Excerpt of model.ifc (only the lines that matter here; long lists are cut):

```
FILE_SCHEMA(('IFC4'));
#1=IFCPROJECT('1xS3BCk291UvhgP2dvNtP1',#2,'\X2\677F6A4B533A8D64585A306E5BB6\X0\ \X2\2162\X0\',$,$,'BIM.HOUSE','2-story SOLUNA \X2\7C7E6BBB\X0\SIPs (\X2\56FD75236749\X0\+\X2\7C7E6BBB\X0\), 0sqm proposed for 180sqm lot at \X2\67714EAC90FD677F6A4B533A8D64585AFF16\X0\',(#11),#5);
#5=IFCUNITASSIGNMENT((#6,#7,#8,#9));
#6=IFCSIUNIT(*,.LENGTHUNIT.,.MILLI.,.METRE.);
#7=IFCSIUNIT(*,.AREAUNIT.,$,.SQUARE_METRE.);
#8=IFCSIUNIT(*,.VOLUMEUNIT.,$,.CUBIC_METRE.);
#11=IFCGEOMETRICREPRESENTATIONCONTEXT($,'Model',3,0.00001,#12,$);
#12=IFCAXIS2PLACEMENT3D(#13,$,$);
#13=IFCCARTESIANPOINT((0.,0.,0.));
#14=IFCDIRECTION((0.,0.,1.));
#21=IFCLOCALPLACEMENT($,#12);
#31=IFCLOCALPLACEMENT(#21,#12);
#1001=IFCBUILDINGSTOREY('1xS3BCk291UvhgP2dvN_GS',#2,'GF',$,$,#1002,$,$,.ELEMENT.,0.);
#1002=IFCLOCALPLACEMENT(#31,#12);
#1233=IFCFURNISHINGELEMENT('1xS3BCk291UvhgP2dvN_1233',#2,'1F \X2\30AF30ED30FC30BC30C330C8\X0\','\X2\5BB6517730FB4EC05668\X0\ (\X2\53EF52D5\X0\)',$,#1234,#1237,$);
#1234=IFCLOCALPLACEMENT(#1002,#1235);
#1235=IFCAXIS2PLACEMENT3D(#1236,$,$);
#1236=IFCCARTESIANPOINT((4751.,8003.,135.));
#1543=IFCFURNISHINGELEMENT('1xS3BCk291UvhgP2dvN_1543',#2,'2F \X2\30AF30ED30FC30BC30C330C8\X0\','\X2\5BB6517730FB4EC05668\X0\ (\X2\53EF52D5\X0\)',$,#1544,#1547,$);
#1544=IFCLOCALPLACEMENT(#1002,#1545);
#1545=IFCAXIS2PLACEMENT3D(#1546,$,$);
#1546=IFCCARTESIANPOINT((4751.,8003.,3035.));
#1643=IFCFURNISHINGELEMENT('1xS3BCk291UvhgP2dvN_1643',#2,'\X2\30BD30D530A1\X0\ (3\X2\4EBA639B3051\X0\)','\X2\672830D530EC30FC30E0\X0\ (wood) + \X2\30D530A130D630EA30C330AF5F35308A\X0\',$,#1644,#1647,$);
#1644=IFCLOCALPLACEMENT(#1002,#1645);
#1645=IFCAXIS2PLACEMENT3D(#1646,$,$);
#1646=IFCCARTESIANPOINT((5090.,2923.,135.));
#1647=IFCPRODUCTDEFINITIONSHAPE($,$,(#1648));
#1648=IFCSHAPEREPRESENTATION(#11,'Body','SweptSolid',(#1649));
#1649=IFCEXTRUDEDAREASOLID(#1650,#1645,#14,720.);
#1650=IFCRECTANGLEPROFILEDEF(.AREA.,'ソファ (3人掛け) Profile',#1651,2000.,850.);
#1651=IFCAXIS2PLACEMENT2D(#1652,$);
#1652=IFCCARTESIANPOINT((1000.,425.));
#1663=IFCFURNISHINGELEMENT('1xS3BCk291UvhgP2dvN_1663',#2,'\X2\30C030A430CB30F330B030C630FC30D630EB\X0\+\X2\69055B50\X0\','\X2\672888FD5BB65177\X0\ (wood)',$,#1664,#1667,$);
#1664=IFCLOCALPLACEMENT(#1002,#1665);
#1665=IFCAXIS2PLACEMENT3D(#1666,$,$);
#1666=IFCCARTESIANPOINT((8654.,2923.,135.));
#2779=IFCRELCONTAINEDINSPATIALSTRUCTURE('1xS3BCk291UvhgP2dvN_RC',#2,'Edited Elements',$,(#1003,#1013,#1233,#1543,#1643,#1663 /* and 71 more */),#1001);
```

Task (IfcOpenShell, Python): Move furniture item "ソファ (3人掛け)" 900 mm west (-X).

```python
import ifcopenshell
import ifcopenshell.api.geometry
import ifcopenshell.util.placement
import ifcopenshell.util.unit

model = ifcopenshell.open("model.ifc")
unit_scale = ifcopenshell.util.unit.calculate_unit_scale(model)

item = model.by_id(1643)
matrix = ifcopenshell.util.placement.get_local_placement(item.ObjectPlacement)
matrix[0, 3] -= 0.9 / unit_scale
ifcopenshell.api.geometry.edit_object_placement(model, product=item, matrix=matrix, is_si=False)

print(ifcopenshell.util.placement.get_local_placement(item.ObjectPlacement).round(3) + 0.0)

model.write("model_updated.ifc")
```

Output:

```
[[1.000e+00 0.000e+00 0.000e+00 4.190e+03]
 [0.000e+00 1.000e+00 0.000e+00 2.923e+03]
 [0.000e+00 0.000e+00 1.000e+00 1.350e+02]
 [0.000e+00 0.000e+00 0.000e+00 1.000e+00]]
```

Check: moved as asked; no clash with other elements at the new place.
